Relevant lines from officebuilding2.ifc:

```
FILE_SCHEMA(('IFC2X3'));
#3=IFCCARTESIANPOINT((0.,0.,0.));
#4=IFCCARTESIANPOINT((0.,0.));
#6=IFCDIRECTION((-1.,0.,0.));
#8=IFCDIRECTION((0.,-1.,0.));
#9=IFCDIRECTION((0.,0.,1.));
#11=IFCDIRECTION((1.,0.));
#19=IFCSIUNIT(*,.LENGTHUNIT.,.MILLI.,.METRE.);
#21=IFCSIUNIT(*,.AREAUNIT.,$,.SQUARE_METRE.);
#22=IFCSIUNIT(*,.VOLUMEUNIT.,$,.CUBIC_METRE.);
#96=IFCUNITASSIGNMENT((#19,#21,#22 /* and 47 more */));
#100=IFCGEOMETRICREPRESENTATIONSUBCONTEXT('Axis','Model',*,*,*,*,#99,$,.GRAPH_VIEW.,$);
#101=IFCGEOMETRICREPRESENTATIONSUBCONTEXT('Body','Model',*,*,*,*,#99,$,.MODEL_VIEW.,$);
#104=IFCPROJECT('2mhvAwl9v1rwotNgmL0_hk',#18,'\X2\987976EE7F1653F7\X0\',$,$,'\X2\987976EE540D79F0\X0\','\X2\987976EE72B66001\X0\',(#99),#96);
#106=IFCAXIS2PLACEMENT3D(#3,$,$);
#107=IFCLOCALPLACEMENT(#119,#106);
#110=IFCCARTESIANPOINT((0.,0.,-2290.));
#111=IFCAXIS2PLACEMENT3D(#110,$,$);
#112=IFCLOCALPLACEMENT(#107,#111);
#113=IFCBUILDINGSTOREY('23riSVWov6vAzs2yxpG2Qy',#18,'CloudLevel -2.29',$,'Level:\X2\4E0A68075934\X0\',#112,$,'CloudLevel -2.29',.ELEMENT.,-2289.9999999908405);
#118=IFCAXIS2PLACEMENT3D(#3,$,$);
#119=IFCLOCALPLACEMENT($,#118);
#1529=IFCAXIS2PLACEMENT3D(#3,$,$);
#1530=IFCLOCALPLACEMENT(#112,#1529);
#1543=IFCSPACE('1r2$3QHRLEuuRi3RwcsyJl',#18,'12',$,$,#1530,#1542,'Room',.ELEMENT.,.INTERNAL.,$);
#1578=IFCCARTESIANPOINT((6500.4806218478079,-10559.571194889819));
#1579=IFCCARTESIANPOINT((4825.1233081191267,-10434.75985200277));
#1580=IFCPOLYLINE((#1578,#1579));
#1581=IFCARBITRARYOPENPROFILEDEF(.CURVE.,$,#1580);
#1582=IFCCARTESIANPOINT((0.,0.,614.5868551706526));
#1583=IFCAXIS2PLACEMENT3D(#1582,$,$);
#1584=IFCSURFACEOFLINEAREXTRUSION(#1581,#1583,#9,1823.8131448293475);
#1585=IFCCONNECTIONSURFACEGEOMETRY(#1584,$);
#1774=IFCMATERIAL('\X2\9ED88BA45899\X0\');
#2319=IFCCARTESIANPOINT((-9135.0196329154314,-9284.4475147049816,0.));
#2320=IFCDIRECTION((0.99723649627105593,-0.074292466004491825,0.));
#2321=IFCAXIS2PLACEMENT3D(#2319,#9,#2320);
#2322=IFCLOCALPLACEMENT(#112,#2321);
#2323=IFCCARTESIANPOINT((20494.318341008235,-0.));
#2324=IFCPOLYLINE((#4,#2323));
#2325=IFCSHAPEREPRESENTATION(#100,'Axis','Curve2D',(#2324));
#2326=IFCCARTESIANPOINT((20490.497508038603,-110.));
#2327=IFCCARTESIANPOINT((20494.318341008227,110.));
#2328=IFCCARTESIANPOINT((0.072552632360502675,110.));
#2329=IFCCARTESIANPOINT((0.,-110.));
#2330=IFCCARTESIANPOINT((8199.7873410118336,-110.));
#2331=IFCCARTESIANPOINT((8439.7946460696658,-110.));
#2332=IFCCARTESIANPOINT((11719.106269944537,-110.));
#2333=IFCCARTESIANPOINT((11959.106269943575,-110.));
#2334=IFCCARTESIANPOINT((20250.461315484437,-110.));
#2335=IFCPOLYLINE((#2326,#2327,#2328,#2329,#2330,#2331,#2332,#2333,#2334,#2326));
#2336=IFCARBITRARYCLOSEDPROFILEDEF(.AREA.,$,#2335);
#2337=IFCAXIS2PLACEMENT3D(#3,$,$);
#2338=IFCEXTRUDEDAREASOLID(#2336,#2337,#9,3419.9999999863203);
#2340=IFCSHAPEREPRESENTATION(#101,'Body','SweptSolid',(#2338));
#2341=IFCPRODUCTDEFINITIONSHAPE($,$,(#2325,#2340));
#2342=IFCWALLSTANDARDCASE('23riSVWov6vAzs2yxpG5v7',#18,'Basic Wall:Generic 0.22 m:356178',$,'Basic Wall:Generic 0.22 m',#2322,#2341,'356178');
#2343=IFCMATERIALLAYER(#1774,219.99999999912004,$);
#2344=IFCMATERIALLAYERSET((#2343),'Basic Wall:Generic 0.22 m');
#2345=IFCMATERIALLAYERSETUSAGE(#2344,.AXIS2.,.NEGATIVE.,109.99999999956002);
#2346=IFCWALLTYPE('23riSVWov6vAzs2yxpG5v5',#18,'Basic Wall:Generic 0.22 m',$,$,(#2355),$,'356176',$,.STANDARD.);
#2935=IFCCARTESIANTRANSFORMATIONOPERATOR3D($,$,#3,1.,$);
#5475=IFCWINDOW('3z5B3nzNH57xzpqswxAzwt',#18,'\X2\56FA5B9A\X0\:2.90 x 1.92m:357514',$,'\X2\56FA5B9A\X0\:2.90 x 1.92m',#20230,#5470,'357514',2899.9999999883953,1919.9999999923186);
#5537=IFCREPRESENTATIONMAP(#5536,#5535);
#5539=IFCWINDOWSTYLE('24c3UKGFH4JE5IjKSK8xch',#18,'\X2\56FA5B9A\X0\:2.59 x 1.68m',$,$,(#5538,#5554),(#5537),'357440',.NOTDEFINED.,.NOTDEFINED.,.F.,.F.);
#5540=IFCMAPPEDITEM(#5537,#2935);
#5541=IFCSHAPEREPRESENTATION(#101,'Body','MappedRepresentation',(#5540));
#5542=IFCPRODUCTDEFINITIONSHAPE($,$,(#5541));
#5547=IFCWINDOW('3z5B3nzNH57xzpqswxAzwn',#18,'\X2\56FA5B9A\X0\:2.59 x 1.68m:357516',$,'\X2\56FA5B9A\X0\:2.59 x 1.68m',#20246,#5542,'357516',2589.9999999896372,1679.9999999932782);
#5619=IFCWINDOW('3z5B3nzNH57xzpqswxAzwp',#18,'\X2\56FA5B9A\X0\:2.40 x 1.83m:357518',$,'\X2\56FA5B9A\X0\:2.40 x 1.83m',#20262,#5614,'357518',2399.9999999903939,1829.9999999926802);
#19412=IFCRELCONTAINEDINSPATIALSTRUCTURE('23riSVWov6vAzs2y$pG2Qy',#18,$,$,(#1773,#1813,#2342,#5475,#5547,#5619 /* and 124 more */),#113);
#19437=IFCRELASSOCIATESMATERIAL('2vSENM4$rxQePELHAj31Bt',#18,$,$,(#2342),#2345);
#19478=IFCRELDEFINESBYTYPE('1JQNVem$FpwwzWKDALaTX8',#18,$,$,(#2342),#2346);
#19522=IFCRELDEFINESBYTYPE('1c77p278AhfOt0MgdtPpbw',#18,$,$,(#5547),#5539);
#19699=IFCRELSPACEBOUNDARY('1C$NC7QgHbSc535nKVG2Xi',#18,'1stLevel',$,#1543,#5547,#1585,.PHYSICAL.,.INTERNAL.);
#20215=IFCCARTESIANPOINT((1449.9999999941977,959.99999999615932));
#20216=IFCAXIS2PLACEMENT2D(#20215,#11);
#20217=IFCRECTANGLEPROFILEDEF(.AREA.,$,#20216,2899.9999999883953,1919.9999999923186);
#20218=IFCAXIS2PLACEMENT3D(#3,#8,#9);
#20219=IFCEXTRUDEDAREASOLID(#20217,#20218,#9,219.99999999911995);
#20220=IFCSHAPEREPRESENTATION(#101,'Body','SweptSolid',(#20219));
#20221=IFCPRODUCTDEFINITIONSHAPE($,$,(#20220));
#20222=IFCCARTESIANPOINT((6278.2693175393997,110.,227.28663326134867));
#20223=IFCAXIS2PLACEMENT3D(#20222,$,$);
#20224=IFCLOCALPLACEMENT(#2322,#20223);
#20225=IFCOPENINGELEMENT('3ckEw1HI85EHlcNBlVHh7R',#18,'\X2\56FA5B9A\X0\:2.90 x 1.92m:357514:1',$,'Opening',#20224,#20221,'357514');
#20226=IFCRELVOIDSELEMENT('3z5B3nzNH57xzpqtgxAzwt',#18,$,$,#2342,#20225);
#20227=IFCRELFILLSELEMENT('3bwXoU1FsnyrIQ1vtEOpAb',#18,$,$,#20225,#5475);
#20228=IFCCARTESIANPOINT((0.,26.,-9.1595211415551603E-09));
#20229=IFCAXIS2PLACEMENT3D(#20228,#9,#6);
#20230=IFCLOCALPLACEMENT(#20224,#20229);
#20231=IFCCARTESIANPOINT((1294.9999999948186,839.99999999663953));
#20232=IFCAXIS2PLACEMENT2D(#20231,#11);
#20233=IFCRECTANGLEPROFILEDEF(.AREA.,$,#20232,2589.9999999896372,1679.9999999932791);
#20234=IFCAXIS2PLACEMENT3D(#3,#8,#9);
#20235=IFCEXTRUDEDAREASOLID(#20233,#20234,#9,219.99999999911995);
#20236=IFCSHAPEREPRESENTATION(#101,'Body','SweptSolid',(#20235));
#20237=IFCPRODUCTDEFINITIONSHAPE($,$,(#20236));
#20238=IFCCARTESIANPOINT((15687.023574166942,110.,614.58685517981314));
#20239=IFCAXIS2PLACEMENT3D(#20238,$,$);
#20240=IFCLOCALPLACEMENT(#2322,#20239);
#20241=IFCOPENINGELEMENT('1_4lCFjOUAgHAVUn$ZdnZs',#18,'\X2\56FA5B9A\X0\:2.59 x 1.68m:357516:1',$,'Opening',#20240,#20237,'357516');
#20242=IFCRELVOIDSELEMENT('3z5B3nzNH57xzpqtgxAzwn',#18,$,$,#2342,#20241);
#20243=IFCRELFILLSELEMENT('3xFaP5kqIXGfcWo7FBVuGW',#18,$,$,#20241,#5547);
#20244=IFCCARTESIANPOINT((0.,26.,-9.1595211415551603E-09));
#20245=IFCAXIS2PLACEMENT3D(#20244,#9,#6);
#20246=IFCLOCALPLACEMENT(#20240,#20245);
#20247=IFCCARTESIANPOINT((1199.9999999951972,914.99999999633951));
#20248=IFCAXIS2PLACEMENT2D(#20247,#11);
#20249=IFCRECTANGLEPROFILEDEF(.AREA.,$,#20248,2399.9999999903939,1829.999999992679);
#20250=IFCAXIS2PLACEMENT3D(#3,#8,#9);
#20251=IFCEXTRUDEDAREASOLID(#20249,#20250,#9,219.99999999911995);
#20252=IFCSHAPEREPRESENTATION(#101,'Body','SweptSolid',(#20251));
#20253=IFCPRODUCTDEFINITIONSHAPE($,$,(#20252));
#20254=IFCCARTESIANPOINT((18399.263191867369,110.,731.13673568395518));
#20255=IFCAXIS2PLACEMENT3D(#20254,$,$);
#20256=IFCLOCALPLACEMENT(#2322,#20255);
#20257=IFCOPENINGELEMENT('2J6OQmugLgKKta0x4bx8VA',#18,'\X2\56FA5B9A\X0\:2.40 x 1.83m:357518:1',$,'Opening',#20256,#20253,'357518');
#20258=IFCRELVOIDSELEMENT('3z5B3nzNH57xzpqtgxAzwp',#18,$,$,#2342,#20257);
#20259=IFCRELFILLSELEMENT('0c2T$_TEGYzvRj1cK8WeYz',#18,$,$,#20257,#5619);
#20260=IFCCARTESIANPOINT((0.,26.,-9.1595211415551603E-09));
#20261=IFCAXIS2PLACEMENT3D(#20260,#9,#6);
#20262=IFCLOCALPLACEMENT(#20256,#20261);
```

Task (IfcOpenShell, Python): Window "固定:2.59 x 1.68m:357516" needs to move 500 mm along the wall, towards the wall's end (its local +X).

```python
import numpy as np
import ifcopenshell
import ifcopenshell.api.geometry
import ifcopenshell.util.placement
import ifcopenshell.util.unit

model = ifcopenshell.open("officebuilding2.ifc")
unit_scale = ifcopenshell.util.unit.calculate_unit_scale(model)

window = model.by_guid("3z5B3nzNH57xzpqswxAzwn")
opening = window.FillsVoids[0].RelatingOpeningElement
wall = opening.VoidsElements[0].RelatingBuildingElement

wall_matrix = ifcopenshell.util.placement.get_local_placement(wall.ObjectPlacement)
shift = wall_matrix[:3, 0] * 0.5 / unit_scale
before = ifcopenshell.util.placement.get_local_placement(window.ObjectPlacement)[:3, 3].copy()

# The window is placed relative to its opening, so it follows when the opening moves.
matrix = ifcopenshell.util.placement.get_local_placement(opening.ObjectPlacement)
matrix[:3, 3] += shift
ifcopenshell.api.geometry.edit_object_placement(
    model, product=opening, matrix=matrix, is_si=False, should_transform_children=True
)

# Space boundary surfaces are stored in each space's coordinates; move them too.
for rel in window.ProvidesBoundaries:
    if not rel.ConnectionGeometry:
        continue
    surface = rel.ConnectionGeometry.SurfaceOnRelatingElement
    space_matrix = ifcopenshell.util.placement.get_local_placement(rel.RelatingSpace.ObjectPlacement)
    point = np.array(surface.Position.Location.Coordinates) + space_matrix[:3, :3].T @ shift
    surface.Position = model.createIfcAxis2Placement3D(
        model.createIfcCartesianPoint(point.tolist()), surface.Position.Axis, surface.Position.RefDirection
    )

after = ifcopenshell.util.placement.get_local_placement(window.ObjectPlacement)[:3, 3]
print("window moved by", (after - before).round(3) + 0.0)

model.write("officebuilding2_rev.ifc")
```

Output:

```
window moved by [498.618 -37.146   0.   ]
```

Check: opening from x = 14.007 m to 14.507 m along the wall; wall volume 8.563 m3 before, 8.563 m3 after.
